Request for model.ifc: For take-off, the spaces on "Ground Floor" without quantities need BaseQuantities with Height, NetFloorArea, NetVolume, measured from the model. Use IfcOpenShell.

First a look at what the model holds.

```python
import ifcopenshell
import ifcopenshell.util.element
import ifcopenshell.util.unit

model = ifcopenshell.open("model.ifc")
print(model.schema)
for unit_type in ("LENGTHUNIT", "AREAUNIT", "VOLUMEUNIT"):
    print(unit_type, ifcopenshell.util.unit.calculate_unit_scale(model, unit_type))
storey = next(s for s in model.by_type("IfcBuildingStorey") if s.Name == "Ground Floor")
spaces = [e for e in ifcopenshell.util.element.get_decomposition(storey) if e.is_a("IfcSpace")]
for e in sorted(spaces, key=lambda e: e.id()):
    print(e.id(), e.is_a(), e.Name, list(ifcopenshell.util.element.get_psets(e, qtos_only=True)), sep=" | ")
```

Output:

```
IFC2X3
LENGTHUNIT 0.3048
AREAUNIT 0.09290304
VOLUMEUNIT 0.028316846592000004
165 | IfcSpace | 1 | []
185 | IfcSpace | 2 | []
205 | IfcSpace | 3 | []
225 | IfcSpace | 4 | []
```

```python
import ifcopenshell
import ifcopenshell.api.pset
import ifcopenshell.geom
import ifcopenshell.util.element
import ifcopenshell.util.shape
import ifcopenshell.util.unit

model = ifcopenshell.open("model.ifc")
unit_scale = ifcopenshell.util.unit.calculate_unit_scale(model)
area_scale = ifcopenshell.util.unit.calculate_unit_scale(model, "AREAUNIT")
volume_scale = ifcopenshell.util.unit.calculate_unit_scale(model, "VOLUMEUNIT")
settings = ifcopenshell.geom.settings()

storey = next(s for s in model.by_type("IfcBuildingStorey") if s.Name == "Ground Floor")
spaces = [e for e in ifcopenshell.util.element.get_decomposition(storey) if e.is_a("IfcSpace")]

for e in sorted(spaces, key=lambda e: e.id()):
    if ifcopenshell.util.element.get_psets(e, qtos_only=True, should_inherit=False):
        continue
    # Geometry comes back in metres, in the element's own axes.
    shape = ifcopenshell.geom.create_shape(settings, e)
    values = {
        "Height": ifcopenshell.util.shape.get_z(shape.geometry) / unit_scale,
        "NetFloorArea": ifcopenshell.util.shape.get_footprint_area(shape.geometry) / area_scale,
        "NetVolume": ifcopenshell.util.shape.get_volume(shape.geometry) / volume_scale,
    }
    qto = ifcopenshell.api.pset.add_qto(model, product=e, name="BaseQuantities")
    ifcopenshell.api.pset.edit_qto(model, qto=qto, properties=values)
    print(e.id(), {k: round(v, 3) for k, v in values.items()})

model.write("model_edited.ifc")
```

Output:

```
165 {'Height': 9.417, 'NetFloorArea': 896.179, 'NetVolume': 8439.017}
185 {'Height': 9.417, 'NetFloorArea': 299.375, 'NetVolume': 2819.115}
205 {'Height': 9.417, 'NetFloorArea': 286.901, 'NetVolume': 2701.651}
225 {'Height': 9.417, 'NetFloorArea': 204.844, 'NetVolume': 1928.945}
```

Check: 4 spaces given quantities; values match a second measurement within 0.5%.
